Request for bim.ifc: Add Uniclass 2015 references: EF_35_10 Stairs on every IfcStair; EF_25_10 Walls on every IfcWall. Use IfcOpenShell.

First a look at what the model holds.

```python
import ifcopenshell

model = ifcopenshell.open("bim.ifc")
print(model.schema)
print("classifications:", [c.Name for c in model.by_type("IfcClassification")])
for ifc_class in ("IfcDoor", "IfcRoof", "IfcStair", "IfcWall", "IfcWindow"):
    print(ifc_class, len(model.by_type(ifc_class)))
```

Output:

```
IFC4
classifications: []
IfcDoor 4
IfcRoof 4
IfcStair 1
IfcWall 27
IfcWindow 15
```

```python
import ifcopenshell
import ifcopenshell.api.classification

model = ifcopenshell.open("bim.ifc")

system = ifcopenshell.api.classification.add_classification(model, classification="Uniclass 2015")

codes = {
    "IfcStair": ("EF_35_10", "Stairs"),
    "IfcWall": ("EF_25_10", "Walls"),
}
for ifc_class, (code, name) in codes.items():
    products = model.by_type(ifc_class)
    ifcopenshell.api.classification.add_reference(
        model, products=products, classification=system, identification=code, name=name
    )
    print(code, len(products))

model.write("bim_v2.ifc")
```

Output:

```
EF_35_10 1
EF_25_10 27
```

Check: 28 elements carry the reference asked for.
